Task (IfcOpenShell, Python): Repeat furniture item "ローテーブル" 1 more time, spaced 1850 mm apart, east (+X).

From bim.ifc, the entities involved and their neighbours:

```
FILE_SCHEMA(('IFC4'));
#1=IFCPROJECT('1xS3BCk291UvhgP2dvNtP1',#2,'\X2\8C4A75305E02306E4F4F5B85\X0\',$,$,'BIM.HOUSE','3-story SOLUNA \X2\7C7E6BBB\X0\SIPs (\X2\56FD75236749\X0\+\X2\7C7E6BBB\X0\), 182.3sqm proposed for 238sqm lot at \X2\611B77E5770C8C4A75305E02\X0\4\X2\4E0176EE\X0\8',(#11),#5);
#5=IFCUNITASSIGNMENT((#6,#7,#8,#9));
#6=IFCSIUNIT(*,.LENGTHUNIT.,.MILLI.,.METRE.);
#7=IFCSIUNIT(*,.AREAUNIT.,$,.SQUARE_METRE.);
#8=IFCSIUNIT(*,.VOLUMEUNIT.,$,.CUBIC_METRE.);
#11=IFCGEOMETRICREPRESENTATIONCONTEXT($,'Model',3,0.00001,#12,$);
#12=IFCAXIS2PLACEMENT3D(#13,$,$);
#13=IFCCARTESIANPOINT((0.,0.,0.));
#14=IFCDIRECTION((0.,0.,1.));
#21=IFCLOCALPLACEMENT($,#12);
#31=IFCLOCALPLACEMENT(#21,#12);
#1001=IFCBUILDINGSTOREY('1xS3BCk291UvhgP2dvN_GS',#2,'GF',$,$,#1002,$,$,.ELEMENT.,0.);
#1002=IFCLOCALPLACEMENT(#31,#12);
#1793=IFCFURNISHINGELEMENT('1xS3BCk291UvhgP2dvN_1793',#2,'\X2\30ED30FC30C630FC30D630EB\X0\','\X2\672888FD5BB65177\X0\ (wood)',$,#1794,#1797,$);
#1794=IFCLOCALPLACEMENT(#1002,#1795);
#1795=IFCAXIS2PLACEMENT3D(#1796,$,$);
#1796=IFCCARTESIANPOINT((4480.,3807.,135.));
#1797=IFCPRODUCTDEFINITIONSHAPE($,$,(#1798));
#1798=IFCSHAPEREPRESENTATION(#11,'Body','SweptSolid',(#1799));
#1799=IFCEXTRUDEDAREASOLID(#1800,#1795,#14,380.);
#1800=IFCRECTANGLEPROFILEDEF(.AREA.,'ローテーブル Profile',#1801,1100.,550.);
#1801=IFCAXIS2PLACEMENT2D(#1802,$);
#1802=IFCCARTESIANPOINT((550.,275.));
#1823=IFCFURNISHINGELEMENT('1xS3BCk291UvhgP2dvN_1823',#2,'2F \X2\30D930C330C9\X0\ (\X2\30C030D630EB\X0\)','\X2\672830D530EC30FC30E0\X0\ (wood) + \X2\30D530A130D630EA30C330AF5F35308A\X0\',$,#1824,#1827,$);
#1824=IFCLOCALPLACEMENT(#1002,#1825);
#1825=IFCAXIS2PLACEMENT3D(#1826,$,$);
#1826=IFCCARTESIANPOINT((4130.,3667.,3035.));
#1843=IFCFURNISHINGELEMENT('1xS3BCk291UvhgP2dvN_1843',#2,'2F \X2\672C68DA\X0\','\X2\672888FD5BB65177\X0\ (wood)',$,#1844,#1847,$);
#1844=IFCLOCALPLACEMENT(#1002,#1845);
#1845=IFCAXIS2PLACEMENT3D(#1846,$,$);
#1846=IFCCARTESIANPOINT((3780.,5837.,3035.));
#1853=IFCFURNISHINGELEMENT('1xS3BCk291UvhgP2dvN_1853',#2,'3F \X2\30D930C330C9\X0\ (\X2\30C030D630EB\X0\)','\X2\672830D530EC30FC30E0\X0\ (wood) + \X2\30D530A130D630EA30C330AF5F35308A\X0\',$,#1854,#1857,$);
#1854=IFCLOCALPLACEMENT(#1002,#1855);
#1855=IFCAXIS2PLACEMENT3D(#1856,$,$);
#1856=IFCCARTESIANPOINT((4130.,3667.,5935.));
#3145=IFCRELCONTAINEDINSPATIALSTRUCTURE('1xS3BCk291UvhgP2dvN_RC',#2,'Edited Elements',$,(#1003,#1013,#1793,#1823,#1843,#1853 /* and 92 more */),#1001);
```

```python
import numpy as np
import ifcopenshell
import ifcopenshell.api.geometry
import ifcopenshell.api.root
import ifcopenshell.util.element
import ifcopenshell.util.placement
import ifcopenshell.util.unit

model = ifcopenshell.open("bim.ifc")
unit_scale = ifcopenshell.util.unit.calculate_unit_scale(model)


def reuse_history(source, copy):
    """copy_class also copies each property set's owner history, people and application; keep the originals."""
    for rel in copy.IsDefinedBy:
        if rel.is_a("IfcRelDefinesByProperties") and (history := rel.RelatingPropertyDefinition.OwnerHistory):
            rel.RelatingPropertyDefinition.OwnerHistory = source.OwnerHistory
            ifcopenshell.util.element.remove_deep2(model, history)


source = model.by_guid("1xS3BCk291UvhgP2dvN_1793")
base = ifcopenshell.util.placement.get_local_placement(source.ObjectPlacement)
step = np.array([1.0, 0.0, 0.0]) * 1.85 / unit_scale

for i in range(1, 2):
    copy = ifcopenshell.api.root.copy_class(model, product=source)
    copy.Representation = ifcopenshell.util.element.copy_deep(
        model, source.Representation, exclude=["IfcGeometricRepresentationContext", "IfcRepresentationMap"]
    )
    reuse_history(source, copy)
    matrix = base.copy()
    matrix[:3, 3] += i * step
    print("added at", matrix[:3, 3].round(3) + 0.0)
    ifcopenshell.api.geometry.edit_object_placement(model, product=copy, matrix=matrix, is_si=False)

model.write("bim_rev.ifc")
```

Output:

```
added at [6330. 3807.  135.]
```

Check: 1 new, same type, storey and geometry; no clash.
